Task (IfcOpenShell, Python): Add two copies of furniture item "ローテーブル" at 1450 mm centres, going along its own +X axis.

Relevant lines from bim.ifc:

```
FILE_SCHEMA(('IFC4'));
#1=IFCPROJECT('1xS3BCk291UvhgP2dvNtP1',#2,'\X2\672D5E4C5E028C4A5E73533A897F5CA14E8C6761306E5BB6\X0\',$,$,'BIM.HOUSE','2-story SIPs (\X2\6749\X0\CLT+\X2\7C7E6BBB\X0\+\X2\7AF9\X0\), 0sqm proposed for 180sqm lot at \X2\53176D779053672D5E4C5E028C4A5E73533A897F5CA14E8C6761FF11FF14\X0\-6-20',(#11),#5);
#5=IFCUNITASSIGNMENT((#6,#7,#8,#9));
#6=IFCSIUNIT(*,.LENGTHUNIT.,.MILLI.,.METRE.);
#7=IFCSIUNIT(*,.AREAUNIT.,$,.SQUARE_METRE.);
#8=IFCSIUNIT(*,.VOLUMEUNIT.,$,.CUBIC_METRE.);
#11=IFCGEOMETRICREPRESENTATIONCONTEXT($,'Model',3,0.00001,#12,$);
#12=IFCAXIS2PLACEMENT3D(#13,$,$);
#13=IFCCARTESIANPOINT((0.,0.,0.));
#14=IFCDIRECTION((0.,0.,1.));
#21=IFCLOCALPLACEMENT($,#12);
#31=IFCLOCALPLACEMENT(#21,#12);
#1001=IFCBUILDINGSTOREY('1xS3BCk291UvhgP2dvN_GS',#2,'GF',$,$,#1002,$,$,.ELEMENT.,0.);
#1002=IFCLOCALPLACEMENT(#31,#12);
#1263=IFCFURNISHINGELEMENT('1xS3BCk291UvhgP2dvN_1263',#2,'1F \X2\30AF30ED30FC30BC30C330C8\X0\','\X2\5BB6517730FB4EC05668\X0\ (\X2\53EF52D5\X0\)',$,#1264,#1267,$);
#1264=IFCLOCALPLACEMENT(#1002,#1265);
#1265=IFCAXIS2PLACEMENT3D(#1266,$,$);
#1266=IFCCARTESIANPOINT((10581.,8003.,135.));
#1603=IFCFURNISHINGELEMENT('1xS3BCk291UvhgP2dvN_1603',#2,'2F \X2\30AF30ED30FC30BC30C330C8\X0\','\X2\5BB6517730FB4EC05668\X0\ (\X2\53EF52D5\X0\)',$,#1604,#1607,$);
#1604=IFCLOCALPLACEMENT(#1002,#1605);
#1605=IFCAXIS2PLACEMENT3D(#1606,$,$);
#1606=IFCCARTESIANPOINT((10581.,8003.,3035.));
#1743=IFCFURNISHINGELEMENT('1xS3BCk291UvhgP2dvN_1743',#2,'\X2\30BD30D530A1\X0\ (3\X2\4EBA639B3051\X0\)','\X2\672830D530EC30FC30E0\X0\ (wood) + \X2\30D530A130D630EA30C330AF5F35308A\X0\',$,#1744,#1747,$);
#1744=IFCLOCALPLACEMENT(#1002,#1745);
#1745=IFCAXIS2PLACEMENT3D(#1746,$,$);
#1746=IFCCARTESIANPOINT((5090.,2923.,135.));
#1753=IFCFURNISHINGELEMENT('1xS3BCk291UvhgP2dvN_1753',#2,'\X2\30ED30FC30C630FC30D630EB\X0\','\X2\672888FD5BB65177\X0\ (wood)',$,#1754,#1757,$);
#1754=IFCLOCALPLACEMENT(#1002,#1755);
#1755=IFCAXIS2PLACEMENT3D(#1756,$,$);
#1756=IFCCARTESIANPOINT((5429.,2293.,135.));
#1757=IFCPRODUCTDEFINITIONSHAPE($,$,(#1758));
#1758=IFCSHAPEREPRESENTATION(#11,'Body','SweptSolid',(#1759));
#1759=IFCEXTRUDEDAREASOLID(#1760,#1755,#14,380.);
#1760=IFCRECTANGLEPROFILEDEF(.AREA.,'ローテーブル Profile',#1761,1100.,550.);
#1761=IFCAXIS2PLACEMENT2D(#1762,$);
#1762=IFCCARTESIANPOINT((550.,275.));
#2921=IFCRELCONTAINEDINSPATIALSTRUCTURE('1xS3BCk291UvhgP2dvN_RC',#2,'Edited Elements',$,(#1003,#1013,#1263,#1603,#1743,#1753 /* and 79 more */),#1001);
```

```python
import ifcopenshell
import ifcopenshell.api.geometry
import ifcopenshell.api.root
import ifcopenshell.util.element
import ifcopenshell.util.placement

model = ifcopenshell.open("bim.ifc")


def reuse_history(source, copy):
    """copy_class also copies each property set's owner history, people and application; keep the originals."""
    for rel in copy.IsDefinedBy:
        if rel.is_a("IfcRelDefinesByProperties") and (history := rel.RelatingPropertyDefinition.OwnerHistory):
            rel.RelatingPropertyDefinition.OwnerHistory = source.OwnerHistory
            ifcopenshell.util.element.remove_deep2(model, history)


source = model.by_id(1753)
base = ifcopenshell.util.placement.get_local_placement(source.ObjectPlacement)
step = base[:3, 0] * 1450.0

for i in range(1, 3):
    copy = ifcopenshell.api.root.copy_class(model, product=source)
    copy.Representation = ifcopenshell.util.element.copy_deep(
        model, source.Representation, exclude=["IfcGeometricRepresentationContext", "IfcRepresentationMap"]
    )
    reuse_history(source, copy)
    matrix = base.copy()
    matrix[:3, 3] += i * step
    print("added at", matrix[:3, 3].round(3) + 0.0)
    ifcopenshell.api.geometry.edit_object_placement(model, product=copy, matrix=matrix, is_si=False)

model.write("bim_v2.ifc")
```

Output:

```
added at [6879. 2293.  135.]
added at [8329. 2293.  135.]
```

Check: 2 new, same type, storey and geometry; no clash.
